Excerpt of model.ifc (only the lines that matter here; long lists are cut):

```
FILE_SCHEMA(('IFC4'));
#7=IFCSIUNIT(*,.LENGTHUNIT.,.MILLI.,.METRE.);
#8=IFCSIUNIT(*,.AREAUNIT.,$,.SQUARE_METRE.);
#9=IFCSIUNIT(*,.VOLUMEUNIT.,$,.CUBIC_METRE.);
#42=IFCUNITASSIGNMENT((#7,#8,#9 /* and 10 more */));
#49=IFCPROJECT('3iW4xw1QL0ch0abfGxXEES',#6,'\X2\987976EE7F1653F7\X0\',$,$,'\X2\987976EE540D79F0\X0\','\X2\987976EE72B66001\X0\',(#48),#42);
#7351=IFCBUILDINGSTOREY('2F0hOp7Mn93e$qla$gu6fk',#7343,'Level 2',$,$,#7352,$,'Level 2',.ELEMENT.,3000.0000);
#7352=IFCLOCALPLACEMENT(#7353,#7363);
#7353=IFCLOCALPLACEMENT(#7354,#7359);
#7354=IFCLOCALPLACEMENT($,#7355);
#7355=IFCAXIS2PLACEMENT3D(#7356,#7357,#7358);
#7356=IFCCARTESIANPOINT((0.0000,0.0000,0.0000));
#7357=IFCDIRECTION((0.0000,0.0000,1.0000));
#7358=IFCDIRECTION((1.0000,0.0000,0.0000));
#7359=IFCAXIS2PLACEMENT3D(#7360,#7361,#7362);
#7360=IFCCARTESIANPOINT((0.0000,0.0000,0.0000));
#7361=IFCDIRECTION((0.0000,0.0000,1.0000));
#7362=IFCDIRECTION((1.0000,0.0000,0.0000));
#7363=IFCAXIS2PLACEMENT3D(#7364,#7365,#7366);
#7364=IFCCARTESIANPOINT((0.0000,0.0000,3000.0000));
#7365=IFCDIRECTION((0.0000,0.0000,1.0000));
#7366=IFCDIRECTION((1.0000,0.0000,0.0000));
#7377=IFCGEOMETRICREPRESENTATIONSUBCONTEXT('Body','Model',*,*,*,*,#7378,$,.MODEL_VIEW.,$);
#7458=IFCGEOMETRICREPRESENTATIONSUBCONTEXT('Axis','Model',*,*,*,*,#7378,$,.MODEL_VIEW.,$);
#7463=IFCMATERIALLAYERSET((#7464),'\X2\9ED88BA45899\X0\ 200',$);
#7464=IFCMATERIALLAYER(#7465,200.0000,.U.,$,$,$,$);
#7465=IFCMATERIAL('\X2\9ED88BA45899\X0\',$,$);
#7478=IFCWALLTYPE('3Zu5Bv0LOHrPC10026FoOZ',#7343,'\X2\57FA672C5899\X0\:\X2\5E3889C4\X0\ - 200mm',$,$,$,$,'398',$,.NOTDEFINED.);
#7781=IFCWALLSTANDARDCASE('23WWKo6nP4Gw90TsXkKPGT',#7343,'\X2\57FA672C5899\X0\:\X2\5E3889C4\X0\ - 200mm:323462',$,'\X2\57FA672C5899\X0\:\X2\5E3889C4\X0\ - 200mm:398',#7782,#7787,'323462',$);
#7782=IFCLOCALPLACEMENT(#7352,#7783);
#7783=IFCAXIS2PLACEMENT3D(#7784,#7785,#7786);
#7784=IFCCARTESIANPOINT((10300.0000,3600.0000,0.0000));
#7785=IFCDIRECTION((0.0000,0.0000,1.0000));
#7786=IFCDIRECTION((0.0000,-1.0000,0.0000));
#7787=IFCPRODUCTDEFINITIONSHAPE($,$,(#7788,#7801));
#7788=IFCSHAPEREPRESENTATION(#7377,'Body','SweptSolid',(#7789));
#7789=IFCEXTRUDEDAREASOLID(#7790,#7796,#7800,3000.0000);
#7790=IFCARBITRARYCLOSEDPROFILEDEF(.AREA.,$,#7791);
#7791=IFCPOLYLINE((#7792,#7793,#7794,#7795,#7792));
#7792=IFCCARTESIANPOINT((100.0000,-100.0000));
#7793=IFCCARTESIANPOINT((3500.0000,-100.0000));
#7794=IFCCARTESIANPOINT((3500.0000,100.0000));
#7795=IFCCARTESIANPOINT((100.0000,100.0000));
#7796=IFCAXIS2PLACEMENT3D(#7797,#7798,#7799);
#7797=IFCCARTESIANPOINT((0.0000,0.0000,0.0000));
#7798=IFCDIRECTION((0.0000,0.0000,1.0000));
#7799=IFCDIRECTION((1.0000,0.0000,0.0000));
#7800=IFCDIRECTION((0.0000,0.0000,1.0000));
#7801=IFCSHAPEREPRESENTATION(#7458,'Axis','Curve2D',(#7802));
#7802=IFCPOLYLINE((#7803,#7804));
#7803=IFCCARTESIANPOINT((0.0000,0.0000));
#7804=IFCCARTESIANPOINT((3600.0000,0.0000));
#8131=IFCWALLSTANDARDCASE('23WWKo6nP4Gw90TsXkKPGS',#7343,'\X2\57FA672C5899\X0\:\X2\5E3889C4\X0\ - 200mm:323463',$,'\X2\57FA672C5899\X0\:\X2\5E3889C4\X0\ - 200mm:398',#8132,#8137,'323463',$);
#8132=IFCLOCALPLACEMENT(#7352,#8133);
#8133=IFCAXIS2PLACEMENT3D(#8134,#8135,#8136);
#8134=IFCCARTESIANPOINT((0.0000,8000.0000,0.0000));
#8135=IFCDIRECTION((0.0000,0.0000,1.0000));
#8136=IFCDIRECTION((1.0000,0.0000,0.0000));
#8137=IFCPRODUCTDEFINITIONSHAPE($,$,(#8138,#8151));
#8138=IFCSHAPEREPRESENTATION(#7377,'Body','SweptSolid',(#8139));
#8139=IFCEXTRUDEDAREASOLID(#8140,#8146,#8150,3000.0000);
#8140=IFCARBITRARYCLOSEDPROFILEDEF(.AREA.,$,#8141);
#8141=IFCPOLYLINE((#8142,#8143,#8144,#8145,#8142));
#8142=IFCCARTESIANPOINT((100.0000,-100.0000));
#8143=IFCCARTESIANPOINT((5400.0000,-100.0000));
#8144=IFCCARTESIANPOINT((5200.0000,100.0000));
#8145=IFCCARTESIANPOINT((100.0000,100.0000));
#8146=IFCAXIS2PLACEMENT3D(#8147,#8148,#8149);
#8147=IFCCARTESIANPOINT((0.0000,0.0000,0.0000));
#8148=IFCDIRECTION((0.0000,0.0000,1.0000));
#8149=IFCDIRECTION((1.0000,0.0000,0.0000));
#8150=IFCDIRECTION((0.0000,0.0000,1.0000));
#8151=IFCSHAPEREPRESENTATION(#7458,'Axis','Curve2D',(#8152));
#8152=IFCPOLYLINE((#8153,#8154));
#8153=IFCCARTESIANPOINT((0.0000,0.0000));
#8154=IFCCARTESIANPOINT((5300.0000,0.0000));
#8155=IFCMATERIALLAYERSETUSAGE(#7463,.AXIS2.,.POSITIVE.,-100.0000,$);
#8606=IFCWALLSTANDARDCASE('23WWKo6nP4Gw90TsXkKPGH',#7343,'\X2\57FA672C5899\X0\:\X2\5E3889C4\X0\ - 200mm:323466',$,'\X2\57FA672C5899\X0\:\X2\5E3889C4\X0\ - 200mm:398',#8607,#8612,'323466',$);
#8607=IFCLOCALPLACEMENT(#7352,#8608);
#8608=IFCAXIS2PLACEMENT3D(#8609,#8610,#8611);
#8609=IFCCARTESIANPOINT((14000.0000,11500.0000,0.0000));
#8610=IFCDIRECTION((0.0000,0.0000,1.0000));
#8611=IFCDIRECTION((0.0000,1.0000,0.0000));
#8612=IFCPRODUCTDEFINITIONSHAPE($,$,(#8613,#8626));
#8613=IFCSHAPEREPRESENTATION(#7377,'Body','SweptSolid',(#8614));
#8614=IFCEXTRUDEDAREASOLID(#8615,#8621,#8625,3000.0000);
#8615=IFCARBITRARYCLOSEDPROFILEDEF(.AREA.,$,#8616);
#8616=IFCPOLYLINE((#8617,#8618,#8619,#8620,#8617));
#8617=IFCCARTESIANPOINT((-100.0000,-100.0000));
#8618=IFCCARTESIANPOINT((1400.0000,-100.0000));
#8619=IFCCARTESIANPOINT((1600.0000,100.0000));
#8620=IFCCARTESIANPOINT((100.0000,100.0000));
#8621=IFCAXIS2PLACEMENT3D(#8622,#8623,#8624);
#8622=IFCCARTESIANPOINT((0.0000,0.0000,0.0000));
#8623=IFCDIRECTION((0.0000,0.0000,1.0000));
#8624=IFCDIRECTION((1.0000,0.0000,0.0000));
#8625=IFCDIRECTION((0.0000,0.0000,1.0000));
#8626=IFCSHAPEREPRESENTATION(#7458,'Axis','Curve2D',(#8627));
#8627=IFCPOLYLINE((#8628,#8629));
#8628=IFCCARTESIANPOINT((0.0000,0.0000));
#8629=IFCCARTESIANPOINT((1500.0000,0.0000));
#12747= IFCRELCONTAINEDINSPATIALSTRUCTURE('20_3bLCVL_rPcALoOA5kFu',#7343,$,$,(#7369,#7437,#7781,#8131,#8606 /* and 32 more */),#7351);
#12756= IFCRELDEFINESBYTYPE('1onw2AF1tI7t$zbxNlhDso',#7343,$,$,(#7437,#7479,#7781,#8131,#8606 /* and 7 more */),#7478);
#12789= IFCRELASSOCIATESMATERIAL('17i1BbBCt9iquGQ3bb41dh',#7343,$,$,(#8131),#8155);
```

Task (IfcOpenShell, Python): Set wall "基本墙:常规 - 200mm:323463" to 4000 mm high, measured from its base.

```python
import ifcopenshell
import ifcopenshell.geom
import ifcopenshell.util.representation
import ifcopenshell.util.shape
import ifcopenshell.util.unit

model = ifcopenshell.open("model.ifc")
unit_scale = ifcopenshell.util.unit.calculate_unit_scale(model)
settings = ifcopenshell.geom.settings()


def volume(element):
    """Net volume in cubic metres, openings subtracted."""
    shape = ifcopenshell.geom.create_shape(settings, element)
    return ifcopenshell.util.shape.get_volume(shape.geometry)


wall = model.by_guid("23WWKo6nP4Gw90TsXkKPGS")
before = volume(wall)

body = ifcopenshell.util.representation.get_representation(wall, "Model", "Body")
solid = body.Items[0]
old_height = solid.Depth
solid.Depth = 4 / unit_scale
after = volume(wall)

print(f"height {old_height:g} -> {solid.Depth:g}, volume {before:.3f} -> {after:.3f} m3")

model.write("model_edited.ifc")
```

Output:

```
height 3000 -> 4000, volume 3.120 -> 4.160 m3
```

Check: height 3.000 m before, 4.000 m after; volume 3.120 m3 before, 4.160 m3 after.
